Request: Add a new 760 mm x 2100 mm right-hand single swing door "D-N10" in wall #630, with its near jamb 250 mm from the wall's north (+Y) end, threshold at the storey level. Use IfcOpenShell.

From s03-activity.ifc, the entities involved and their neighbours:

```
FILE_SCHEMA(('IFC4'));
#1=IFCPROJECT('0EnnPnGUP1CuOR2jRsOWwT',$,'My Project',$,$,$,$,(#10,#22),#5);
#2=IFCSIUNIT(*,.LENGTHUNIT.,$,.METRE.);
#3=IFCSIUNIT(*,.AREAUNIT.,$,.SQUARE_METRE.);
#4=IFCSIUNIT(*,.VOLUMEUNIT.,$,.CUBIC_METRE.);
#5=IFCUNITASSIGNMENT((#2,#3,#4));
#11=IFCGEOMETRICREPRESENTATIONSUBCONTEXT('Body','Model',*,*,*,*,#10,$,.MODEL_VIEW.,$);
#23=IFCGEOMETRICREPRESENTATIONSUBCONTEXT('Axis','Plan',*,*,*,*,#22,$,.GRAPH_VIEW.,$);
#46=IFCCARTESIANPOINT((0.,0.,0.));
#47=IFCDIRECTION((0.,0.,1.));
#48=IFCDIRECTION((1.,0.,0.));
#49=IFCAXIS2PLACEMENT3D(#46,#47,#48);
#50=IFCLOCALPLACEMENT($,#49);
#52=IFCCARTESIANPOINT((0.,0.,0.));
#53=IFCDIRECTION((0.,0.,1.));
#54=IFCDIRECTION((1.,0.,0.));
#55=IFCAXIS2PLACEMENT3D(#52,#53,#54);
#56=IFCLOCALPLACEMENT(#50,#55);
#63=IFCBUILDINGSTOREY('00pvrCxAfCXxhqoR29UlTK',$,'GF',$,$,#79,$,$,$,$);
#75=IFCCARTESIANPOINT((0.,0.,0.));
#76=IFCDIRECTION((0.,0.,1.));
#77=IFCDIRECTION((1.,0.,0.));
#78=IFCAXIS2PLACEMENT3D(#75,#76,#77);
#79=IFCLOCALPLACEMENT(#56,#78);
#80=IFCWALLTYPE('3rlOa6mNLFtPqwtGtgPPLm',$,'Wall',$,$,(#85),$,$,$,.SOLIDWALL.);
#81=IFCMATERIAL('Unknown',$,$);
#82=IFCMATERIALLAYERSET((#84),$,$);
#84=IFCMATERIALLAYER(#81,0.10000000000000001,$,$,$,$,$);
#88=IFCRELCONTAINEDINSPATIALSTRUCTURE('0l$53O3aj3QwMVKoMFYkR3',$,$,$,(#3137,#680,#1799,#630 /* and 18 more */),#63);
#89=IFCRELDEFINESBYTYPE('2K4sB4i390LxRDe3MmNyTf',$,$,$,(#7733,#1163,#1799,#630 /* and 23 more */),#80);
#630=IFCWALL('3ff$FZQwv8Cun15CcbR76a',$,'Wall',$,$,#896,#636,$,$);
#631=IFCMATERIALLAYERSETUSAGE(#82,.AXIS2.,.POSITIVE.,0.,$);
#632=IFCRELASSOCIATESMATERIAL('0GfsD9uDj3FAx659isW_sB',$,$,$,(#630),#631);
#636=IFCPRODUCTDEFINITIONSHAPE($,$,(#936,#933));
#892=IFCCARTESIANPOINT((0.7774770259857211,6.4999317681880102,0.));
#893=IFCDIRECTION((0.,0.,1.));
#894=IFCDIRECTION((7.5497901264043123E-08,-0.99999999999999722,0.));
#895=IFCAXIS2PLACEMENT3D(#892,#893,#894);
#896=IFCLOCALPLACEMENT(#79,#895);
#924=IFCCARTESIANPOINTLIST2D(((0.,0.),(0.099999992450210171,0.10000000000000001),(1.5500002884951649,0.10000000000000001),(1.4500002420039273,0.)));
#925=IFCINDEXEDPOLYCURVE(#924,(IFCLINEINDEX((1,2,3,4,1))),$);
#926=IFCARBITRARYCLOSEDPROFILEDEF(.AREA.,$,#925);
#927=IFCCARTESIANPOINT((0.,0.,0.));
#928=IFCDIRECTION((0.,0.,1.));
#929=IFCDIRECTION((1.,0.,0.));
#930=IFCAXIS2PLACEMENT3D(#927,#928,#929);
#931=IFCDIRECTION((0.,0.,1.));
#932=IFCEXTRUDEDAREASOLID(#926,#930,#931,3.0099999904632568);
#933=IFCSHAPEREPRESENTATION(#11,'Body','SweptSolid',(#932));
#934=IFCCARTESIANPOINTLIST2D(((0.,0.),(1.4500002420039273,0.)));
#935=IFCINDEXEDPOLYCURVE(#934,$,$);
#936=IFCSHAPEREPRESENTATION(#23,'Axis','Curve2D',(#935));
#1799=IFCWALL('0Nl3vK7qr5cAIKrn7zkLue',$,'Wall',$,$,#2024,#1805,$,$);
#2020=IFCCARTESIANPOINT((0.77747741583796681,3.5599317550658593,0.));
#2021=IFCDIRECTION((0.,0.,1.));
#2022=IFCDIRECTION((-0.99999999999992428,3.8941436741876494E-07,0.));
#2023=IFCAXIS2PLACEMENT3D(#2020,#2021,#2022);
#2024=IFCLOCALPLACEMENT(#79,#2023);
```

```python
import numpy as np
import ifcopenshell
import ifcopenshell.api.feature
import ifcopenshell.api.geometry
import ifcopenshell.api.root
import ifcopenshell.api.spatial
import ifcopenshell.geom
import ifcopenshell.util.element
import ifcopenshell.util.placement
import ifcopenshell.util.representation
import ifcopenshell.util.shape
import ifcopenshell.util.unit

model = ifcopenshell.open("s03-activity.ifc")
unit_scale = ifcopenshell.util.unit.calculate_unit_scale(model)
settings = ifcopenshell.geom.settings()


def volume(element):
    """Net volume in cubic metres, openings subtracted."""
    shape = ifcopenshell.geom.create_shape(settings, element)
    return ifcopenshell.util.shape.get_volume(shape.geometry)


wall = model.by_guid("3ff$FZQwv8Cun15CcbR76a")
storey = ifcopenshell.util.element.get_container(wall, ifc_class="IfcBuildingStorey")
context = ifcopenshell.util.representation.get_context(model, "Model", "Body", "MODEL_VIEW")
before = volume(wall)

width, height, from_end, sill = 0.76, 2.1, 0.25, 0.0  # metres

# The wall runs along its own X axis, and the end named is its -X end.
wall_shape = ifcopenshell.geom.create_shape(settings, wall)
x, y, z = ifcopenshell.util.shape.get_vertices(wall_shape.geometry).T
start = x.min() + from_end
face, thickness = float(y.min()), float(y.max() - y.min())
wall_matrix = ifcopenshell.util.placement.get_local_placement(wall.ObjectPlacement)
level = ifcopenshell.util.placement.get_local_placement(storey.ObjectPlacement)[2, 3]


def in_wall(x, y):
    """Placement at x, y metres in the wall's axes, at sill height."""
    matrix = wall_matrix.copy()
    matrix[:, 3] = wall_matrix @ np.array([x / unit_scale, y / unit_scale, 0.0, 1.0])
    matrix[2, 3] = level + sill / unit_scale
    return matrix


# Opening: a box that overshoots both wall faces by 50 mm.
opening = ifcopenshell.api.root.create_entity(model, ifc_class="IfcOpeningElement", predefined_type="OPENING")
box = ifcopenshell.api.geometry.add_wall_representation(
    model, context=context, length=width, height=height, thickness=thickness + 0.1
)
ifcopenshell.api.geometry.assign_representation(model, product=opening, representation=box)
ifcopenshell.api.geometry.edit_object_placement(model, product=opening, matrix=in_wall(start, face - 0.05), is_si=False)
ifcopenshell.api.feature.add_feature(model, feature=opening, element=wall)

door = ifcopenshell.api.root.create_entity(model, ifc_class="IfcDoor", name="D-N10", predefined_type="DOOR")
door.OverallWidth, door.OverallHeight = width / unit_scale, height / unit_scale
door.OperationType = "SINGLE_SWING_RIGHT"
body = ifcopenshell.api.geometry.add_door_representation(
    model,
    context=context,
    overall_width=door.OverallWidth,
    overall_height=door.OverallHeight,
    operation_type="SINGLE_SWING_RIGHT",
    lining_properties={"LiningDepth": thickness / unit_scale, "ThresholdDepth": thickness / unit_scale},
)
ifcopenshell.api.geometry.assign_representation(model, product=door, representation=body)
ifcopenshell.api.spatial.assign_container(model, products=[door], relating_structure=storey)
ifcopenshell.api.feature.add_filling(model, opening=opening, element=door)

# The lining spans the wall, so the door starts at the wall face.
ifcopenshell.api.geometry.edit_object_placement(model, product=door, matrix=in_wall(start, face), is_si=False)

after = volume(wall)

print(f"wall volume {before:.3f} -> {after:.3f} m3")

model.write("s03-activity-out.ifc")
```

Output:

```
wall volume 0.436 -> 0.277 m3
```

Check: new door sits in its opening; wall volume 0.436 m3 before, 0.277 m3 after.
